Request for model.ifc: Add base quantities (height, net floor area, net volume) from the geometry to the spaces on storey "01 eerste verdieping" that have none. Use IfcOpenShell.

First a look at what the model holds.

```python
import ifcopenshell
import ifcopenshell.util.element
import ifcopenshell.util.unit

model = ifcopenshell.open("model.ifc")
print(model.schema)
for unit_type in ("LENGTHUNIT", "AREAUNIT", "VOLUMEUNIT"):
    print(unit_type, ifcopenshell.util.unit.calculate_unit_scale(model, unit_type))
storey = next(s for s in model.by_type("IfcBuildingStorey") if s.Name == "01 eerste verdieping")
spaces = [e for e in ifcopenshell.util.element.get_decomposition(storey) if e.is_a("IfcSpace")]
for e in sorted(spaces, key=lambda e: e.id()):
    print(e.id(), e.is_a(), e.Name, list(ifcopenshell.util.element.get_psets(e, qtos_only=True)), sep=" | ")
```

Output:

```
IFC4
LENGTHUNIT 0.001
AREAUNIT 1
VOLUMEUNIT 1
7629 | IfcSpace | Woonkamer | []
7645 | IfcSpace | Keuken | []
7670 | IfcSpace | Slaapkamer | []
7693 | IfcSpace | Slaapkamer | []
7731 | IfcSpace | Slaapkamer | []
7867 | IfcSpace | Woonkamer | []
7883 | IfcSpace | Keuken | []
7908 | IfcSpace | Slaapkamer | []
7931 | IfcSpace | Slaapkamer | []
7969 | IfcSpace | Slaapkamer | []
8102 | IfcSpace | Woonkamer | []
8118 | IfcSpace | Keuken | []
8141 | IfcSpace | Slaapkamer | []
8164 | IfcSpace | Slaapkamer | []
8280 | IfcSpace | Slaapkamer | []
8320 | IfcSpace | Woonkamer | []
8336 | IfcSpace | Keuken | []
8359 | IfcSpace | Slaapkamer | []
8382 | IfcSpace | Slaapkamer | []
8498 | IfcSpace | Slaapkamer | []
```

```python
import ifcopenshell
import ifcopenshell.api.pset
import ifcopenshell.geom
import ifcopenshell.util.element
import ifcopenshell.util.shape
import ifcopenshell.util.unit

model = ifcopenshell.open("model.ifc")
unit_scale = ifcopenshell.util.unit.calculate_unit_scale(model)
area_scale = ifcopenshell.util.unit.calculate_unit_scale(model, "AREAUNIT")
volume_scale = ifcopenshell.util.unit.calculate_unit_scale(model, "VOLUMEUNIT")
settings = ifcopenshell.geom.settings()

storey = next(s for s in model.by_type("IfcBuildingStorey") if s.Name == "01 eerste verdieping")
spaces = [e for e in ifcopenshell.util.element.get_decomposition(storey) if e.is_a("IfcSpace")]

for e in sorted(spaces, key=lambda e: e.id()):
    if ifcopenshell.util.element.get_psets(e, qtos_only=True, should_inherit=False):
        continue
    # Geometry comes back in metres, in the element's own axes.
    shape = ifcopenshell.geom.create_shape(settings, e)
    values = {
        "Height": ifcopenshell.util.shape.get_z(shape.geometry) / unit_scale,
        "NetFloorArea": ifcopenshell.util.shape.get_footprint_area(shape.geometry) / area_scale,
        "NetVolume": ifcopenshell.util.shape.get_volume(shape.geometry) / volume_scale,
    }
    qto = ifcopenshell.api.pset.add_qto(model, product=e, name="Qto_SpaceBaseQuantities")
    ifcopenshell.api.pset.edit_qto(model, qto=qto, properties=values)
    print(e.id(), {k: round(v, 3) for k, v in values.items()})

model.write("model-out.ifc")
```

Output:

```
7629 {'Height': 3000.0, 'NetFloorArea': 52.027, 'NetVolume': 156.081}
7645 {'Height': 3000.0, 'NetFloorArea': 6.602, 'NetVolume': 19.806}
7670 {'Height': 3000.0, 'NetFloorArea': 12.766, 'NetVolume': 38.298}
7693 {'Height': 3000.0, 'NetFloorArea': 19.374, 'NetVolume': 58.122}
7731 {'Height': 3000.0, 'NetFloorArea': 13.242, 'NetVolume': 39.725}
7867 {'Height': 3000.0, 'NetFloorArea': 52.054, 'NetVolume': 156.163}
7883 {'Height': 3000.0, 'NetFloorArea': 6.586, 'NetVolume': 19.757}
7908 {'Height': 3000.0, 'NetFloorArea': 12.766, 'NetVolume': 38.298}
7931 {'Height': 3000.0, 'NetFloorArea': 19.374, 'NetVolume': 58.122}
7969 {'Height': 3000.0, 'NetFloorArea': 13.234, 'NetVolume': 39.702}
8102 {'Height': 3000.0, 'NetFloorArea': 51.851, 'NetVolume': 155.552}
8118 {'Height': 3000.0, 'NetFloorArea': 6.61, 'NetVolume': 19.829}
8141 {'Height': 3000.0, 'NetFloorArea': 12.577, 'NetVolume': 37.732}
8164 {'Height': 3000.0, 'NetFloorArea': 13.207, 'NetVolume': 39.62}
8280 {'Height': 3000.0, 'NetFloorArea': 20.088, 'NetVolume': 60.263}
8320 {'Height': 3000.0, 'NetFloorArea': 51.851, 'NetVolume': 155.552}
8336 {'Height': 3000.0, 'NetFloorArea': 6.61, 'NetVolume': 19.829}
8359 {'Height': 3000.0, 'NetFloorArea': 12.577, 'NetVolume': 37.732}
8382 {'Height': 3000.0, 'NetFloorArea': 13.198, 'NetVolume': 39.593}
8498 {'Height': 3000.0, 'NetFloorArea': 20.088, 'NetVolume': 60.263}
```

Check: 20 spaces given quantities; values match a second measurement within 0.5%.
